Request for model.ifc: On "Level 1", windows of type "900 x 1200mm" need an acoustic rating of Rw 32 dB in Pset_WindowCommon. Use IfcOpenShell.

First a look at what the model holds.

```python
import ifcopenshell
import ifcopenshell.util.element

model = ifcopenshell.open("model.ifc")
print(model.schema)
storey = next(s for s in model.by_type("IfcBuildingStorey") if s.Name == "Level 1")
windows = [e for e in ifcopenshell.util.element.get_decomposition(storey) if e.is_a("IfcWindow")]
seen = {}
for e in windows:
    element_type = ifcopenshell.util.element.get_type(e)
    key = (element_type.Name if element_type != e and element_type else None, ifcopenshell.util.element.get_pset(e, "Pset_WindowCommon", "AcousticRating"))
    seen[key] = seen.get(key, 0) + 1
for (name, value), count in sorted(seen.items(), key=str):
    print(count, "x", name, "|", value)
```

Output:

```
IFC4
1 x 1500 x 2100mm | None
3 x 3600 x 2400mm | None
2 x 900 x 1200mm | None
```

```python
import ifcopenshell
import ifcopenshell.api.pset
import ifcopenshell.util.element

model = ifcopenshell.open("model.ifc")

storey = next(s for s in model.by_type("IfcBuildingStorey") if s.Name == "Level 1")
windows = [e for e in ifcopenshell.util.element.get_decomposition(storey) if e.is_a("IfcWindow")]

count = 0
for e in windows:
    element_type = ifcopenshell.util.element.get_type(e)
    if element_type in (None, e) or element_type.Name != "900 x 1200mm":
        continue
    # add_pset returns the element's existing set when there is one.
    pset = ifcopenshell.api.pset.add_pset(model, product=e, name="Pset_WindowCommon")
    ifcopenshell.api.pset.edit_pset(model, pset=pset, properties={"AcousticRating": "Rw 32 dB"})
    count += 1

print(count, "windows updated")

model.write("model_v2.ifc")
```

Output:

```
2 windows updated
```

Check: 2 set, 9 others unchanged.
